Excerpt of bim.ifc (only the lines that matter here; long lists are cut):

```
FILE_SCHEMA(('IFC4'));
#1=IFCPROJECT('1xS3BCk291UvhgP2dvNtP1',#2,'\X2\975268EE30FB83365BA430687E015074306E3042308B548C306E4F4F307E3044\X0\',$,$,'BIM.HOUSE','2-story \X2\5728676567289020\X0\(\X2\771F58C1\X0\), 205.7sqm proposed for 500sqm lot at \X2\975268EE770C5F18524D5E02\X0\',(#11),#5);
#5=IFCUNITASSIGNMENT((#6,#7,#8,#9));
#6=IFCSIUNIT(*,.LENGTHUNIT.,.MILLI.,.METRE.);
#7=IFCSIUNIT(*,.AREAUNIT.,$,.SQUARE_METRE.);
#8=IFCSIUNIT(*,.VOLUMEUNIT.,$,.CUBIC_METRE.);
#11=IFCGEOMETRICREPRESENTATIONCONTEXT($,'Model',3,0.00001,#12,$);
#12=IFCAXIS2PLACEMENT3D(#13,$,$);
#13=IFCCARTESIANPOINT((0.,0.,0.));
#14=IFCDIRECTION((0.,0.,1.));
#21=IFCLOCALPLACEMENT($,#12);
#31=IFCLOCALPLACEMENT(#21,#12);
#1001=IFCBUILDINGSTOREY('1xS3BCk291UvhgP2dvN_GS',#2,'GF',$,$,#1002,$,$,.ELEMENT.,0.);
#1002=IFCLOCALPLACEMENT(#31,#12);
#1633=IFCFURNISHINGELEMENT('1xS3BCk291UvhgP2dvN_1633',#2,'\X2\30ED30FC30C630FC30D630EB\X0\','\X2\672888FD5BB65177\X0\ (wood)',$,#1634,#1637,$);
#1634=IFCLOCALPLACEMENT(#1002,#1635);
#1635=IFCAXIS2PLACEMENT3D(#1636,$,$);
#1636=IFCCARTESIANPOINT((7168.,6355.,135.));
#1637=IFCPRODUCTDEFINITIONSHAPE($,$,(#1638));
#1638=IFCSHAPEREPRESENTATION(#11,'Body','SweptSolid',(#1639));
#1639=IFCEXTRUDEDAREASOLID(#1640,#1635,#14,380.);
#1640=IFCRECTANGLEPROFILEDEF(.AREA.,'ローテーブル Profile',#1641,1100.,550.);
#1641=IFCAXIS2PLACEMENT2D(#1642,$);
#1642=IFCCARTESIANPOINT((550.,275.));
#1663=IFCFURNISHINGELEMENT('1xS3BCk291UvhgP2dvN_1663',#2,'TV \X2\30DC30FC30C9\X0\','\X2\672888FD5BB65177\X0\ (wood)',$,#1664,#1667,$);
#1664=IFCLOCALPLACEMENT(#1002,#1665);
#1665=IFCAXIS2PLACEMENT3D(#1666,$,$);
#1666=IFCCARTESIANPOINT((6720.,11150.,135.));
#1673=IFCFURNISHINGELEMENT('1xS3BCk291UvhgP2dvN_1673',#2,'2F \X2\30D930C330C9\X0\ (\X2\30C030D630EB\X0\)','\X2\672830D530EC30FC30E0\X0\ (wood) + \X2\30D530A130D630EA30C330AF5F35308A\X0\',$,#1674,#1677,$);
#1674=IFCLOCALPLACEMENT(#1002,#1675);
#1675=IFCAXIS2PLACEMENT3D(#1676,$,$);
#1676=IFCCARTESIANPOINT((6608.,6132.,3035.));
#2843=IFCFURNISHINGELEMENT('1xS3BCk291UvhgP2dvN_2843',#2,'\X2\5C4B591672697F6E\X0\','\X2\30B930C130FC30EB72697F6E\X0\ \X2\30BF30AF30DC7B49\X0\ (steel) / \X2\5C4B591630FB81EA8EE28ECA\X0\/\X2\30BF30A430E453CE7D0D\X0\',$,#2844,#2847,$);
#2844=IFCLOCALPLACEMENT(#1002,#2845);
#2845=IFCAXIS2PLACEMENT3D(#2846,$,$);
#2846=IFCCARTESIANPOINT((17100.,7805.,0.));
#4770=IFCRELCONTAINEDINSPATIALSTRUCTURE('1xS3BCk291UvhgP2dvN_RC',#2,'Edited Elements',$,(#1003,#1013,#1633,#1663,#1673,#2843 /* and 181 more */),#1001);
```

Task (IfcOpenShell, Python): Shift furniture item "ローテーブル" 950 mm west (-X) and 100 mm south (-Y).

```python
import ifcopenshell
import ifcopenshell.api.geometry
import ifcopenshell.util.placement

model = ifcopenshell.open("bim.ifc")

item = model.by_id(1633)
matrix = ifcopenshell.util.placement.get_local_placement(item.ObjectPlacement)
matrix[0, 3] -= 950.0
matrix[1, 3] -= 100.0
ifcopenshell.api.geometry.edit_object_placement(model, product=item, matrix=matrix, is_si=False)

print(ifcopenshell.util.placement.get_local_placement(item.ObjectPlacement).round(3) + 0.0)

model.write("bim_v2.ifc")
```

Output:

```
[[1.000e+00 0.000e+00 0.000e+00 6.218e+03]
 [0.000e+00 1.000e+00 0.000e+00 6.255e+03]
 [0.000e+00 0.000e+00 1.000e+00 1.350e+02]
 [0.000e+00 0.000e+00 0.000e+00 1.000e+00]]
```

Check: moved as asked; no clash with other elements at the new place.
